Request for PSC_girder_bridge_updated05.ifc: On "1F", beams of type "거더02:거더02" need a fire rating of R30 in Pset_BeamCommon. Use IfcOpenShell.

First a look at what the model holds.

```python
import ifcopenshell
import ifcopenshell.util.element

model = ifcopenshell.open("PSC_girder_bridge_updated05.ifc")
print(model.schema)
storey = next(s for s in model.by_type("IfcBuildingStorey") if s.Name == "1F")
beams = [e for e in ifcopenshell.util.element.get_decomposition(storey) if e.is_a("IfcBeam")]
seen = {}
for e in beams:
    element_type = ifcopenshell.util.element.get_type(e)
    key = (element_type.Name if element_type != e and element_type else None, ifcopenshell.util.element.get_pset(e, "Pset_BeamCommon", "FireRating"))
    seen[key] = seen.get(key, 0) + 1
for (name, value), count in sorted(seen.items(), key=str):
    print(count, "x", name, "|", value)
```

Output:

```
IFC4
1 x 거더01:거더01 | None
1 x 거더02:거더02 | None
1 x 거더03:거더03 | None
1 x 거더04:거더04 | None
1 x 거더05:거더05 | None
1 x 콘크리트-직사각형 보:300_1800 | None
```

```python
import ifcopenshell
import ifcopenshell.api.pset
import ifcopenshell.util.element

model = ifcopenshell.open("PSC_girder_bridge_updated05.ifc")

storey = next(s for s in model.by_type("IfcBuildingStorey") if s.Name == "1F")
beams = [e for e in ifcopenshell.util.element.get_decomposition(storey) if e.is_a("IfcBeam")]

count = 0
for e in beams:
    element_type = ifcopenshell.util.element.get_type(e)
    if element_type in (None, e) or element_type.Name != "거더02:거더02":
        continue
    # add_pset returns the element's existing set when there is one.
    pset = ifcopenshell.api.pset.add_pset(model, product=e, name="Pset_BeamCommon")
    ifcopenshell.api.pset.edit_pset(model, pset=pset, properties={"FireRating": "R30"})
    count += 1

print(count, "beams updated")

model.write("PSC_girder_bridge_updated05_edited.ifc")
```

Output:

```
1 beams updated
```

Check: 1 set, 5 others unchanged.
